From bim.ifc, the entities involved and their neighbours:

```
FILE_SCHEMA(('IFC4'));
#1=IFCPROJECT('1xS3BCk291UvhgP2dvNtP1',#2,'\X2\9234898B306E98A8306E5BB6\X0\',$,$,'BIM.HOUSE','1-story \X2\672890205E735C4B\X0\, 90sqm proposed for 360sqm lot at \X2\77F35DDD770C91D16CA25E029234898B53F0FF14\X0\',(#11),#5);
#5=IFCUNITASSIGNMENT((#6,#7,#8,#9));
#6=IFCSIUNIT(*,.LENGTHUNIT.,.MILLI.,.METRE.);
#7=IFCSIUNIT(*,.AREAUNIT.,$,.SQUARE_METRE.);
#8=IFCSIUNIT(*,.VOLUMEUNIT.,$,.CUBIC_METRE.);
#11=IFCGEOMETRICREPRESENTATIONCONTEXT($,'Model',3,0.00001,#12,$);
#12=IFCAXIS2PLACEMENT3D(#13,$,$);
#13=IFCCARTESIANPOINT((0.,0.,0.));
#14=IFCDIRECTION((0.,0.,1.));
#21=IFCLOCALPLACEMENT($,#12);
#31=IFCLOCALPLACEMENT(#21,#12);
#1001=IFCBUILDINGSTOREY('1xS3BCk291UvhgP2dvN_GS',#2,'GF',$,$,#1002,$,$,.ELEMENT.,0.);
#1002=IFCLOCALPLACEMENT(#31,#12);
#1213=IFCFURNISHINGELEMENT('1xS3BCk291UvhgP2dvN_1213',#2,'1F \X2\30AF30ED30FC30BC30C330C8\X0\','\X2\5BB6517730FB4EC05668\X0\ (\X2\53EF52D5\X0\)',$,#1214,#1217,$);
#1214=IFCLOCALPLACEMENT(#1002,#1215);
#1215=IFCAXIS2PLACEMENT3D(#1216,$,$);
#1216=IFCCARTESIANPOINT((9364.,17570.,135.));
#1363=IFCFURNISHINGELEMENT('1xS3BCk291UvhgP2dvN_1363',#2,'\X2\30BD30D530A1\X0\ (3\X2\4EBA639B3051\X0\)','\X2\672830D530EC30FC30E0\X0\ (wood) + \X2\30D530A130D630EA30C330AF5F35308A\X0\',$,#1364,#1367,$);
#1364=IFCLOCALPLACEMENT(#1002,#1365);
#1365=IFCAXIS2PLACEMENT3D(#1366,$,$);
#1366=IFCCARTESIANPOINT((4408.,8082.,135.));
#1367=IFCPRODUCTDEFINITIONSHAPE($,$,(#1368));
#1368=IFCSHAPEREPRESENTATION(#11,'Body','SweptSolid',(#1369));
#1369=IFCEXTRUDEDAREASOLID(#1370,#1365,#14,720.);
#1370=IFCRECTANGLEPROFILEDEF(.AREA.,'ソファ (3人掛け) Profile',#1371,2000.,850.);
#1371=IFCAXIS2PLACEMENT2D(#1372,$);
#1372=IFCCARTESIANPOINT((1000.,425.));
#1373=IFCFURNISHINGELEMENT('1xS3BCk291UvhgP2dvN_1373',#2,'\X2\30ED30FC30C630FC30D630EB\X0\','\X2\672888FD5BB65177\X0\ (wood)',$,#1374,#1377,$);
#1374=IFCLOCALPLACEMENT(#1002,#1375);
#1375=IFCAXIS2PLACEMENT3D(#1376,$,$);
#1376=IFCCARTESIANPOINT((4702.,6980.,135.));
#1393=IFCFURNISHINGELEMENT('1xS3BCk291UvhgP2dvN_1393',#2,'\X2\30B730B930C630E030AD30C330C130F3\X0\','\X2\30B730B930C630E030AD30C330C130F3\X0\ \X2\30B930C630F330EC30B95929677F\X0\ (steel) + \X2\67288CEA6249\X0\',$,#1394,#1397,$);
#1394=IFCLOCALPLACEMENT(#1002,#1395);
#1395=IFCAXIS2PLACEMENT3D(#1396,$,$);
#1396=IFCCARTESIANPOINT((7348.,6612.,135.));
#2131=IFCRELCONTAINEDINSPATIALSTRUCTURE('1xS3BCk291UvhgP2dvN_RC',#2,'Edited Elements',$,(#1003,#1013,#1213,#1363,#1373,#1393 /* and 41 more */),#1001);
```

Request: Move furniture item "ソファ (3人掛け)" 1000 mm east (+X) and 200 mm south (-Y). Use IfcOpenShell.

```python
import ifcopenshell
import ifcopenshell.api.geometry
import ifcopenshell.util.placement
import ifcopenshell.util.unit

model = ifcopenshell.open("bim.ifc")
unit_scale = ifcopenshell.util.unit.calculate_unit_scale(model)

item = model.by_guid("1xS3BCk291UvhgP2dvN_1363")
matrix = ifcopenshell.util.placement.get_local_placement(item.ObjectPlacement)
matrix[0, 3] += 1 / unit_scale
matrix[1, 3] -= 0.2 / unit_scale
ifcopenshell.api.geometry.edit_object_placement(model, product=item, matrix=matrix, is_si=False)

print(ifcopenshell.util.placement.get_local_placement(item.ObjectPlacement).round(3) + 0.0)

model.write("bim_rev.ifc")
```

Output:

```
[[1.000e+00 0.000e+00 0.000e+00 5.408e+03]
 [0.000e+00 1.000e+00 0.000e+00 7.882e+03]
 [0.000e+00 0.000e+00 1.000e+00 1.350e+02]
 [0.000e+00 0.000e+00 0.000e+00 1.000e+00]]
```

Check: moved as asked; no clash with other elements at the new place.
